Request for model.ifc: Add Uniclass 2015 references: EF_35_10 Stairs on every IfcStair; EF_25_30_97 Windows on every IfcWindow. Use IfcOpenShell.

First a look at what the model holds.

```python
import ifcopenshell

model = ifcopenshell.open("model.ifc")
print(model.schema)
print("classifications:", [c.Name for c in model.by_type("IfcClassification")])
for ifc_class in ("IfcDoor", "IfcRoof", "IfcStair", "IfcWall", "IfcWindow"):
    print(ifc_class, len(model.by_type(ifc_class)))
```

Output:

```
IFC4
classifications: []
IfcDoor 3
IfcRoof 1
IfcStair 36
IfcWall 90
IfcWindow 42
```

```python
import ifcopenshell
import ifcopenshell.api.classification

model = ifcopenshell.open("model.ifc")

system = ifcopenshell.api.classification.add_classification(model, classification="Uniclass 2015")

codes = {
    "IfcStair": ("EF_35_10", "Stairs"),
    "IfcWindow": ("EF_25_30_97", "Windows"),
}
for ifc_class, (code, name) in codes.items():
    products = model.by_type(ifc_class)
    ifcopenshell.api.classification.add_reference(
        model, products=products, classification=system, identification=code, name=name
    )
    print(code, len(products))

model.write("model-out.ifc")
```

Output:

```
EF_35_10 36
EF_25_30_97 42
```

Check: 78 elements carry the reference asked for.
